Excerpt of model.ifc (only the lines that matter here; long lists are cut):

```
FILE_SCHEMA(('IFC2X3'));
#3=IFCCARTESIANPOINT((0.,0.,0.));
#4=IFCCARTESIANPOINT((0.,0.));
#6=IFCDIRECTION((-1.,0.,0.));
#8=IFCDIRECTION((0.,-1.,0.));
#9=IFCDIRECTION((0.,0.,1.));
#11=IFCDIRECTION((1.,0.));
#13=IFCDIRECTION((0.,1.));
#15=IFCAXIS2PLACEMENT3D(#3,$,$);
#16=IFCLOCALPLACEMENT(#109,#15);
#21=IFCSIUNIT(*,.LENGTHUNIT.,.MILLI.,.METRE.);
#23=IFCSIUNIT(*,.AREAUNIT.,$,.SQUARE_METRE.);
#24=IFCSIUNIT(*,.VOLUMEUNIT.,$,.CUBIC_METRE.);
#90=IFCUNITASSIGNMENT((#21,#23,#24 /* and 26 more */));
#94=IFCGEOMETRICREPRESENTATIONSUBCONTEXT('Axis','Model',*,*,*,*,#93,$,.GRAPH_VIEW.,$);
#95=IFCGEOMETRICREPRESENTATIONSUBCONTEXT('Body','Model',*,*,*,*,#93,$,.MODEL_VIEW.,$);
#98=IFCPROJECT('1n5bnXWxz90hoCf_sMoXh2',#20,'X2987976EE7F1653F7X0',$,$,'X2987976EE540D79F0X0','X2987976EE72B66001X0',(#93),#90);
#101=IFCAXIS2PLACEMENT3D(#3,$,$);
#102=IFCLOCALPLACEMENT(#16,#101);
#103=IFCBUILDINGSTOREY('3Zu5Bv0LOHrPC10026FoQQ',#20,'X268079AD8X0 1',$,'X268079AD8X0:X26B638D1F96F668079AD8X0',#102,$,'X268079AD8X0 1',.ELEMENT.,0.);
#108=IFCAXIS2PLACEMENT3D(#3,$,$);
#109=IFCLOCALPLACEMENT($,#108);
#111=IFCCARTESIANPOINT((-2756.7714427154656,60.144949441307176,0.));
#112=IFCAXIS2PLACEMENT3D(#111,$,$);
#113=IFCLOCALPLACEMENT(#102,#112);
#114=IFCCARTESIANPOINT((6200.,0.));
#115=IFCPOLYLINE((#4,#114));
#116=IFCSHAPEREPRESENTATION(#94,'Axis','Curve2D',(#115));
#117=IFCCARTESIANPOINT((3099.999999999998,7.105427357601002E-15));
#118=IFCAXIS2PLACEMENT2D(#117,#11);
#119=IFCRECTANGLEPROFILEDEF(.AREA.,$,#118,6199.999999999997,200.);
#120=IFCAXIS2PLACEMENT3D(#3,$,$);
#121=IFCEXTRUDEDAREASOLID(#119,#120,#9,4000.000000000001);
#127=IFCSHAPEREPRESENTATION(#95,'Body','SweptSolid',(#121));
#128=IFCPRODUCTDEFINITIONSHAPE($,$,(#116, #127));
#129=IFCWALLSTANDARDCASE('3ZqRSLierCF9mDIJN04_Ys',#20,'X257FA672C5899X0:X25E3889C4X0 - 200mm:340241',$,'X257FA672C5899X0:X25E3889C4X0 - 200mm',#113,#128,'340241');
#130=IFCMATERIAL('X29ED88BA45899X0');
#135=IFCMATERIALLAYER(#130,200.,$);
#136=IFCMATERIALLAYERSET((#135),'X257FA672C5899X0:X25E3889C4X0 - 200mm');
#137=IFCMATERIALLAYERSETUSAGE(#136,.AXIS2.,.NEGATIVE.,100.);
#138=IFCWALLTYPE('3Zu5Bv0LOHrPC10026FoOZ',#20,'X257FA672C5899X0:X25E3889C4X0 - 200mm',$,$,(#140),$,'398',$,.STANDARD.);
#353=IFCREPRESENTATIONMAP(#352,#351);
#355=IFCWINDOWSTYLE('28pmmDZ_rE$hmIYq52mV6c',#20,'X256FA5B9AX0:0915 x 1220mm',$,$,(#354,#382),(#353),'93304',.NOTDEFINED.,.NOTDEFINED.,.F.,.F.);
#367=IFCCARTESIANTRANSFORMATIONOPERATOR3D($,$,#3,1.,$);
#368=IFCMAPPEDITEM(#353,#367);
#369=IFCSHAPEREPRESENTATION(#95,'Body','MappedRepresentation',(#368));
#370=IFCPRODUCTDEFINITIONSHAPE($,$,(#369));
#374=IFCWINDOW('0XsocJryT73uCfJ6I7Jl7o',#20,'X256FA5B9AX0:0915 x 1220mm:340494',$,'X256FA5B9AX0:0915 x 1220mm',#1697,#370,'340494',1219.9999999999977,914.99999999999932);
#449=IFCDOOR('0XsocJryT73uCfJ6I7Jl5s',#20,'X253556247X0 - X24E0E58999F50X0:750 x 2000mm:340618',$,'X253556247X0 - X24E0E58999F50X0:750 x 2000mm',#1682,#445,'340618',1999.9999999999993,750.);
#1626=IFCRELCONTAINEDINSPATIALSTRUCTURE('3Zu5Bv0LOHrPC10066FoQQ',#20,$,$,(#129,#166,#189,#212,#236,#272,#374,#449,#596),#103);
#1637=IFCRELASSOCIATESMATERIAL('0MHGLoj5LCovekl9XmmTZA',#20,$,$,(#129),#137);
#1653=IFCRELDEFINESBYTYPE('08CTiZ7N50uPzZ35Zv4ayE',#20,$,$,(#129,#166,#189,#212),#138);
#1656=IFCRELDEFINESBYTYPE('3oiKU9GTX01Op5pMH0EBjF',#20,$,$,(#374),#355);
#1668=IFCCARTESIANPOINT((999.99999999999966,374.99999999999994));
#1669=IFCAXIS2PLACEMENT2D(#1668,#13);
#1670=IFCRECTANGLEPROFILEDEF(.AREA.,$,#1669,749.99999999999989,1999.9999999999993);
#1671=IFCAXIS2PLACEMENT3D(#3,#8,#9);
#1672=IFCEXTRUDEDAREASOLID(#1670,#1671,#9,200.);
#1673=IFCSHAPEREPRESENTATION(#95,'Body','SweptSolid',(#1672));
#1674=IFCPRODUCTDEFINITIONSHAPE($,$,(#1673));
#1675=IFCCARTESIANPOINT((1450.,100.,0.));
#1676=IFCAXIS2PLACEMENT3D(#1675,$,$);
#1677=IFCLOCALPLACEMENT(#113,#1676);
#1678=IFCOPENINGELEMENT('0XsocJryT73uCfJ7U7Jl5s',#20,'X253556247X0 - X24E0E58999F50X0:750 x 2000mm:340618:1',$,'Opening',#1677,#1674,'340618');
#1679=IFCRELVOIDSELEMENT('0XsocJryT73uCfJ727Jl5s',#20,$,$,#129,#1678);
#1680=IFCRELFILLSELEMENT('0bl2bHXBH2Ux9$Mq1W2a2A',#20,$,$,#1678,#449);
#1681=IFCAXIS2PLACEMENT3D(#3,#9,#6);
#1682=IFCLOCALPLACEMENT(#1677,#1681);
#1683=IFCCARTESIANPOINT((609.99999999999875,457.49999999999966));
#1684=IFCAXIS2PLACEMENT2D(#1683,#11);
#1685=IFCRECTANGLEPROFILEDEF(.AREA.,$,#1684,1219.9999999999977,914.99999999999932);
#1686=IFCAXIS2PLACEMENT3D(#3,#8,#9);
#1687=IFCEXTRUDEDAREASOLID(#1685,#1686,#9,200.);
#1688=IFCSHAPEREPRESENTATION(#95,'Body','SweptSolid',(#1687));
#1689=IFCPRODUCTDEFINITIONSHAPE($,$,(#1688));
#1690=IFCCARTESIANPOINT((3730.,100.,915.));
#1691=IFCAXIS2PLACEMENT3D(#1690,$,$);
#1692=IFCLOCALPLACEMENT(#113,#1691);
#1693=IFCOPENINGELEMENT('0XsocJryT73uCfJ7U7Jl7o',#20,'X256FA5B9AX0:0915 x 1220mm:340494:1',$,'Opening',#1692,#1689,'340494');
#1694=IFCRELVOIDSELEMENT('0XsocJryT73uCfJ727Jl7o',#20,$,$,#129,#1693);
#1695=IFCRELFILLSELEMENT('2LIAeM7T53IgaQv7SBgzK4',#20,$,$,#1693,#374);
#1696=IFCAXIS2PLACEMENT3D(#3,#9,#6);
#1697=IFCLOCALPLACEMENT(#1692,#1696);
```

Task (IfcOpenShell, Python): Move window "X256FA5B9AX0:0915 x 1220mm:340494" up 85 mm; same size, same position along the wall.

```python
import numpy as np
import ifcopenshell
import ifcopenshell.api.geometry
import ifcopenshell.util.placement
import ifcopenshell.util.unit

model = ifcopenshell.open("model.ifc")
unit_scale = ifcopenshell.util.unit.calculate_unit_scale(model)

window = model.by_guid("0XsocJryT73uCfJ6I7Jl7o")
opening = window.FillsVoids[0].RelatingOpeningElement
dz = 85.0

shift = np.array([0.0, 0.0, dz])
# The window is placed relative to its opening, so it follows when the opening moves.
matrix = ifcopenshell.util.placement.get_local_placement(opening.ObjectPlacement)
matrix[:3, 3] += shift
ifcopenshell.api.geometry.edit_object_placement(
    model, product=opening, matrix=matrix, is_si=False, should_transform_children=True
)

print(f"moved by {dz * unit_scale:+.3f} m")

model.write("model_v2.ifc")
```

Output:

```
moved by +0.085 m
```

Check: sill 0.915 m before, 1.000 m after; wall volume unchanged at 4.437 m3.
